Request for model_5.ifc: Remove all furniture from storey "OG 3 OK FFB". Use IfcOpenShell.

First a look at what the model holds.

```python
import ifcopenshell
import ifcopenshell.util.element

model = ifcopenshell.open("model_5.ifc")
print(model.schema)
storey = next(s for s in model.by_type("IfcBuildingStorey") if s.Name == "OG 3 OK FFB")
furniture = [e for e in ifcopenshell.util.element.get_decomposition(storey) if e.is_a("IfcFurnishingElement")]
seen = {}
for e in furniture:
    element_type = ifcopenshell.util.element.get_type(e)
    name = element_type.Name if element_type not in (None, e) else None
    seen[name] = seen.get(name, 0) + 1
for name, count in sorted(seen.items(), key=str):
    print(count, "x", name)
```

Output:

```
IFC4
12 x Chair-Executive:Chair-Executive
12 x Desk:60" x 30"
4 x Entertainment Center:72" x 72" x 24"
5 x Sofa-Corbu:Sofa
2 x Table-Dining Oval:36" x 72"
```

```python
import ifcopenshell
import ifcopenshell.api.root
import ifcopenshell.util.element

model = ifcopenshell.open("model_5.ifc")

storey = next(s for s in model.by_type("IfcBuildingStorey") if s.Name == "OG 3 OK FFB")
furniture = [e for e in ifcopenshell.util.element.get_decomposition(storey) if e.is_a("IfcFurnishingElement")]

for e in furniture:
    ifcopenshell.api.root.remove_product(model, product=e)
print(len(furniture), "removed")

model.write("model_5-out.ifc")
```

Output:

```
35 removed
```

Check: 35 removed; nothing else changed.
